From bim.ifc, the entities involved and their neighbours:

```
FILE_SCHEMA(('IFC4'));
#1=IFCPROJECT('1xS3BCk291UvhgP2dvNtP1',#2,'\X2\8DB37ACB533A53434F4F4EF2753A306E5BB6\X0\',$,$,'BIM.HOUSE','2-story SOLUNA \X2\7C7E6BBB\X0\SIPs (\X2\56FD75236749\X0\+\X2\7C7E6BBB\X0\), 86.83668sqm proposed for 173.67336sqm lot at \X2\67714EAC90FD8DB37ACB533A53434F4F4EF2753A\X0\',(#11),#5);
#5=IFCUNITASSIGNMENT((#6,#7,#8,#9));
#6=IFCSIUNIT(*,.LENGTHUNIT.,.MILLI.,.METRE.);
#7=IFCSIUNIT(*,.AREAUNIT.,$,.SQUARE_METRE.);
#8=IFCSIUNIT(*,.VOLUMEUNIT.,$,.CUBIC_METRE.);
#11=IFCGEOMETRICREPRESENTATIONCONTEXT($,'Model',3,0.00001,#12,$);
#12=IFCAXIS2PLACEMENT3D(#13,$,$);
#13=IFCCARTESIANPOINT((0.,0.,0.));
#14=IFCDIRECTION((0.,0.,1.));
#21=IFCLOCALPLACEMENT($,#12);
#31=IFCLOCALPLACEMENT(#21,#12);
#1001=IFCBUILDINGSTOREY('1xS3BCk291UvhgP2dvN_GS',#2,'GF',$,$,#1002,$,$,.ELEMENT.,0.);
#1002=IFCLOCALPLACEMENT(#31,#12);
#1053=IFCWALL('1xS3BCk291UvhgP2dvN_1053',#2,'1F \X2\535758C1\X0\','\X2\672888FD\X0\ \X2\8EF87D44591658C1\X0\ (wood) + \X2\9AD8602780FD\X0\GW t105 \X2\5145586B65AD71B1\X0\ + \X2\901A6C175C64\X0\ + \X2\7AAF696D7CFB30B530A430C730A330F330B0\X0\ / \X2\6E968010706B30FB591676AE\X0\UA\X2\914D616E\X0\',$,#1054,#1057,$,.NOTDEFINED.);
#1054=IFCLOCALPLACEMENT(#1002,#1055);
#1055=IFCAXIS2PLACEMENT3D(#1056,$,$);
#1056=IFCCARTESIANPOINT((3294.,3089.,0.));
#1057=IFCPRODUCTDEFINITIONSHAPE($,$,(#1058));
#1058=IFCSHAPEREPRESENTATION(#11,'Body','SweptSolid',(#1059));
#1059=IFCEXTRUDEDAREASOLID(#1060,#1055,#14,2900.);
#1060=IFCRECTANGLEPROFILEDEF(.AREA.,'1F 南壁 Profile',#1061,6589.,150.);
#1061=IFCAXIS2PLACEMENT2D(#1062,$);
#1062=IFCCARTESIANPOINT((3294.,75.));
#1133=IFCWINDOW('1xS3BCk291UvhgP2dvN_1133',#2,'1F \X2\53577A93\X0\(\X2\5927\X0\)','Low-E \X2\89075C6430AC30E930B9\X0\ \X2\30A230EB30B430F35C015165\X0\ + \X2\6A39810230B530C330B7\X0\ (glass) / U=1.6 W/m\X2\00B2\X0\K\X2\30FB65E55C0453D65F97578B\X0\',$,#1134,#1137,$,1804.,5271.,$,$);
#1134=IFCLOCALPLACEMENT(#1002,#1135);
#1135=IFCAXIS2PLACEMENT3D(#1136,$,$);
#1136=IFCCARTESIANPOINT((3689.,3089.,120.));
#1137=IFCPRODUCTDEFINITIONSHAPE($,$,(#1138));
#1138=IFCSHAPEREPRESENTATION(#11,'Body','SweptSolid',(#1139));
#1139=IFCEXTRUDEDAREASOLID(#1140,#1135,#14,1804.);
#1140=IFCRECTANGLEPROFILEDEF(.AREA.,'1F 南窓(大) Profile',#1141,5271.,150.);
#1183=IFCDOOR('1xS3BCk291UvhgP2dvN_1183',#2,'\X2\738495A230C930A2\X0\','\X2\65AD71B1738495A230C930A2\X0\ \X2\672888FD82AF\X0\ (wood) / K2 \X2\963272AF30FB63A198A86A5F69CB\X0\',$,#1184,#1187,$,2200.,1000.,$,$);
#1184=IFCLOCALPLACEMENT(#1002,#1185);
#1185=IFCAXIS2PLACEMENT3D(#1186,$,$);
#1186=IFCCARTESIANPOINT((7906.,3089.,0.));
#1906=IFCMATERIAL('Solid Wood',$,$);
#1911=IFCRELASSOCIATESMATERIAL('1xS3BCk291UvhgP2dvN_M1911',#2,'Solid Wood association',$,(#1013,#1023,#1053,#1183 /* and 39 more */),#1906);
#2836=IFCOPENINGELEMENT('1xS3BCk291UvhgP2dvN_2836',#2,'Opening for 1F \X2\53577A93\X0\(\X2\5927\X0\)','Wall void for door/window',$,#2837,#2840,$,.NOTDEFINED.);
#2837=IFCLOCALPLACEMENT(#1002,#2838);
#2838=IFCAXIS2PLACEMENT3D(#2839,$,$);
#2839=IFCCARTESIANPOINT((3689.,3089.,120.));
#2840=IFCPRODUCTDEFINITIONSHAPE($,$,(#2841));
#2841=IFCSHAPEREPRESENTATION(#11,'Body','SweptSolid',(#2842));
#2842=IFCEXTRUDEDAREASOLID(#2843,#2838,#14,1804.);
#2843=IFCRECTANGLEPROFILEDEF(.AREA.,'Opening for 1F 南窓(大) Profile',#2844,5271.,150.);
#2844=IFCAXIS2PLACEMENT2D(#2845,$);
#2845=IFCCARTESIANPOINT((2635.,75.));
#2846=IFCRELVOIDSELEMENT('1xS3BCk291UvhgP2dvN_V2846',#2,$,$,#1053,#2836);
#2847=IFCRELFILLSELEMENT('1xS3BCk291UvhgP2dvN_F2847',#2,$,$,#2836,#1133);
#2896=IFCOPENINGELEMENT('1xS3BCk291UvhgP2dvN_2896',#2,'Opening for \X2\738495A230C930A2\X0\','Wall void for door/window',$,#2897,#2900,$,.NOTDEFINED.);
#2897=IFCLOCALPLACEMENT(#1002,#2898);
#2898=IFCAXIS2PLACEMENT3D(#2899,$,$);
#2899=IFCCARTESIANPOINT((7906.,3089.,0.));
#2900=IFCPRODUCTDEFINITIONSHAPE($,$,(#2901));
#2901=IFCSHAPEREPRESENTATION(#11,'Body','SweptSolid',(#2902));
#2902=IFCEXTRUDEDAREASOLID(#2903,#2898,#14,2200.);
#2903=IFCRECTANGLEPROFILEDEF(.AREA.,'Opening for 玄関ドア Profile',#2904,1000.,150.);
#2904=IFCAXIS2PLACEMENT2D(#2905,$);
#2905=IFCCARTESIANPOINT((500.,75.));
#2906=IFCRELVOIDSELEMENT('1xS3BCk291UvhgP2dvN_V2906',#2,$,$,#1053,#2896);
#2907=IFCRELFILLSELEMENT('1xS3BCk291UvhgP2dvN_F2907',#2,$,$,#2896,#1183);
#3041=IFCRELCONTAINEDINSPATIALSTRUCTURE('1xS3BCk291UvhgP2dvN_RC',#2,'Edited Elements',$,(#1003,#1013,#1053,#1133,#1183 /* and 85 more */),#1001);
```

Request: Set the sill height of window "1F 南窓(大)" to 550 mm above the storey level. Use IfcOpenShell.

```python
import numpy as np
import ifcopenshell
import ifcopenshell.api.geometry
import ifcopenshell.geom
import ifcopenshell.util.element
import ifcopenshell.util.placement
import ifcopenshell.util.shape
import ifcopenshell.util.unit

model = ifcopenshell.open("bim.ifc")
unit_scale = ifcopenshell.util.unit.calculate_unit_scale(model)

window = model.by_guid("1xS3BCk291UvhgP2dvN_1133")
opening = window.FillsVoids[0].RelatingOpeningElement
storey = ifcopenshell.util.element.get_container(window, ifc_class="IfcBuildingStorey")
level = ifcopenshell.util.placement.get_local_placement(storey.ObjectPlacement)[2, 3]

# The opening's origin need not be at the sill, so measure its lowest point.
shape = ifcopenshell.geom.create_shape(ifcopenshell.geom.settings(), opening)
bottom = ifcopenshell.util.shape.get_shape_bottom_elevation(shape, shape.geometry) / unit_scale
dz = level + 0.55 / unit_scale - bottom

shift = np.array([0.0, 0.0, dz])
# The window is not placed relative to its opening, so move both.
for product in (opening, window):
    matrix = ifcopenshell.util.placement.get_local_placement(product.ObjectPlacement)
    matrix[:3, 3] += shift
    ifcopenshell.api.geometry.edit_object_placement(model, product=product, matrix=matrix, is_si=False)

print(f"moved by {dz * unit_scale:+.3f} m")

model.write("bim_rev.ifc")
```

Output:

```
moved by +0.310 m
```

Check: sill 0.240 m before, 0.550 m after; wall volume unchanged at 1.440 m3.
